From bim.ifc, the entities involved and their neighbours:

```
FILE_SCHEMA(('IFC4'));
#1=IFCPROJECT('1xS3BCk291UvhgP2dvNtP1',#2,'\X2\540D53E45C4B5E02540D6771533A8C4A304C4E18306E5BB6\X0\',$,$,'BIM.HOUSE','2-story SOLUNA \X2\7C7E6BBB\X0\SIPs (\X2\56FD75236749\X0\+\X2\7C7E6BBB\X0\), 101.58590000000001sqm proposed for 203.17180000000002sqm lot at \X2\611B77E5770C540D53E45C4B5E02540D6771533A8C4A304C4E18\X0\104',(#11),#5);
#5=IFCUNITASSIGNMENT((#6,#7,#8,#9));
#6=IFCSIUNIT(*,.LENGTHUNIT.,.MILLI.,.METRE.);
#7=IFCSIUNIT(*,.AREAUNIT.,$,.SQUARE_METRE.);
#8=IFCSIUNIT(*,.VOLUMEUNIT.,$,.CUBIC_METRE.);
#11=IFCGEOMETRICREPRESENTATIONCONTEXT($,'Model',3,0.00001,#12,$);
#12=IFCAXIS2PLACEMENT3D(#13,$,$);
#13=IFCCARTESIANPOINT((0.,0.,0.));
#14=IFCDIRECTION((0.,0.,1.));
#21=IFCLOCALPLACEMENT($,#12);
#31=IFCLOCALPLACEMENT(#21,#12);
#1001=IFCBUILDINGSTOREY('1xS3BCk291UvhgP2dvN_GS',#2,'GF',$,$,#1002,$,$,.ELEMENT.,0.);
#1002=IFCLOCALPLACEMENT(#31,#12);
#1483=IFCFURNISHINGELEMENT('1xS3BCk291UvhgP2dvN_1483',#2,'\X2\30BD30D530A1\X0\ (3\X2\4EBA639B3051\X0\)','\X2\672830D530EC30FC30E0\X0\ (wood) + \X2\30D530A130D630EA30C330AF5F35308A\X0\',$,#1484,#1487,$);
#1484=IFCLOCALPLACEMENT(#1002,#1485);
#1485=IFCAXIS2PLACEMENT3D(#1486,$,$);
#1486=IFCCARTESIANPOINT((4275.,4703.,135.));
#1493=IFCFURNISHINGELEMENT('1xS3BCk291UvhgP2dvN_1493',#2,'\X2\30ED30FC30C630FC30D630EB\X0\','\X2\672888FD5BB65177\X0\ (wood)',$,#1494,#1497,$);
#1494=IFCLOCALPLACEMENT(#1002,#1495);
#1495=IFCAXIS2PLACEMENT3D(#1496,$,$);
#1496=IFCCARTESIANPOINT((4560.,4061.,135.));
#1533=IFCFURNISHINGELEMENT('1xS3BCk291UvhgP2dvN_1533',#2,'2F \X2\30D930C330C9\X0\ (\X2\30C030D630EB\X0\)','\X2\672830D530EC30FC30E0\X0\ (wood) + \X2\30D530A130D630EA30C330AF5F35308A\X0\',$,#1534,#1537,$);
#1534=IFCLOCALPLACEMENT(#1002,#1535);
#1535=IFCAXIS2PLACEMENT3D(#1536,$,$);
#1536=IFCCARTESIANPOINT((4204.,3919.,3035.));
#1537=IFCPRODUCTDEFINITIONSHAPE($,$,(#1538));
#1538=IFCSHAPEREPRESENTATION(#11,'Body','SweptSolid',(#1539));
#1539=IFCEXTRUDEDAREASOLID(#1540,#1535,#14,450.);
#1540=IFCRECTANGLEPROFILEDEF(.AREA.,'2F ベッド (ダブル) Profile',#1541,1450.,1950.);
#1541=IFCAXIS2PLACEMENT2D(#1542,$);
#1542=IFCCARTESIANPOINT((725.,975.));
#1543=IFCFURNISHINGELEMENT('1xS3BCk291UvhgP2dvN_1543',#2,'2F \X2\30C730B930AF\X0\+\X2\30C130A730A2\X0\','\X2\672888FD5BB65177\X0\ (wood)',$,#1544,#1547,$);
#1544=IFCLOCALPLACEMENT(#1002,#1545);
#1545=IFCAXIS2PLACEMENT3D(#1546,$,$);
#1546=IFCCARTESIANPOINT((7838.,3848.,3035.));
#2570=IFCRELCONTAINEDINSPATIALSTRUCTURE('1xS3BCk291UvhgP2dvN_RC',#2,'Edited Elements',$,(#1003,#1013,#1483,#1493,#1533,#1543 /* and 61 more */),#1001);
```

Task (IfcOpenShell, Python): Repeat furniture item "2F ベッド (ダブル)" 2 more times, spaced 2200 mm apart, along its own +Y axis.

```python
import ifcopenshell
import ifcopenshell.api.geometry
import ifcopenshell.api.root
import ifcopenshell.util.element
import ifcopenshell.util.placement
import ifcopenshell.util.unit

model = ifcopenshell.open("bim.ifc")
unit_scale = ifcopenshell.util.unit.calculate_unit_scale(model)


def reuse_history(source, copy):
    """copy_class also copies each property set's owner history, people and application; keep the originals."""
    for rel in copy.IsDefinedBy:
        if rel.is_a("IfcRelDefinesByProperties") and (history := rel.RelatingPropertyDefinition.OwnerHistory):
            rel.RelatingPropertyDefinition.OwnerHistory = source.OwnerHistory
            ifcopenshell.util.element.remove_deep2(model, history)


source = model.by_guid("1xS3BCk291UvhgP2dvN_1533")
base = ifcopenshell.util.placement.get_local_placement(source.ObjectPlacement)
step = base[:3, 1] * 2.2 / unit_scale

for i in range(1, 3):
    copy = ifcopenshell.api.root.copy_class(model, product=source)
    copy.Representation = ifcopenshell.util.element.copy_deep(
        model, source.Representation, exclude=["IfcGeometricRepresentationContext", "IfcRepresentationMap"]
    )
    reuse_history(source, copy)
    matrix = base.copy()
    matrix[:3, 3] += i * step
    print("added at", matrix[:3, 3].round(3) + 0.0)
    ifcopenshell.api.geometry.edit_object_placement(model, product=copy, matrix=matrix, is_si=False)

model.write("bim_edited.ifc")
```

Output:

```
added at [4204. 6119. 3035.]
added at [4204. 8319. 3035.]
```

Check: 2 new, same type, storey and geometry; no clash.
